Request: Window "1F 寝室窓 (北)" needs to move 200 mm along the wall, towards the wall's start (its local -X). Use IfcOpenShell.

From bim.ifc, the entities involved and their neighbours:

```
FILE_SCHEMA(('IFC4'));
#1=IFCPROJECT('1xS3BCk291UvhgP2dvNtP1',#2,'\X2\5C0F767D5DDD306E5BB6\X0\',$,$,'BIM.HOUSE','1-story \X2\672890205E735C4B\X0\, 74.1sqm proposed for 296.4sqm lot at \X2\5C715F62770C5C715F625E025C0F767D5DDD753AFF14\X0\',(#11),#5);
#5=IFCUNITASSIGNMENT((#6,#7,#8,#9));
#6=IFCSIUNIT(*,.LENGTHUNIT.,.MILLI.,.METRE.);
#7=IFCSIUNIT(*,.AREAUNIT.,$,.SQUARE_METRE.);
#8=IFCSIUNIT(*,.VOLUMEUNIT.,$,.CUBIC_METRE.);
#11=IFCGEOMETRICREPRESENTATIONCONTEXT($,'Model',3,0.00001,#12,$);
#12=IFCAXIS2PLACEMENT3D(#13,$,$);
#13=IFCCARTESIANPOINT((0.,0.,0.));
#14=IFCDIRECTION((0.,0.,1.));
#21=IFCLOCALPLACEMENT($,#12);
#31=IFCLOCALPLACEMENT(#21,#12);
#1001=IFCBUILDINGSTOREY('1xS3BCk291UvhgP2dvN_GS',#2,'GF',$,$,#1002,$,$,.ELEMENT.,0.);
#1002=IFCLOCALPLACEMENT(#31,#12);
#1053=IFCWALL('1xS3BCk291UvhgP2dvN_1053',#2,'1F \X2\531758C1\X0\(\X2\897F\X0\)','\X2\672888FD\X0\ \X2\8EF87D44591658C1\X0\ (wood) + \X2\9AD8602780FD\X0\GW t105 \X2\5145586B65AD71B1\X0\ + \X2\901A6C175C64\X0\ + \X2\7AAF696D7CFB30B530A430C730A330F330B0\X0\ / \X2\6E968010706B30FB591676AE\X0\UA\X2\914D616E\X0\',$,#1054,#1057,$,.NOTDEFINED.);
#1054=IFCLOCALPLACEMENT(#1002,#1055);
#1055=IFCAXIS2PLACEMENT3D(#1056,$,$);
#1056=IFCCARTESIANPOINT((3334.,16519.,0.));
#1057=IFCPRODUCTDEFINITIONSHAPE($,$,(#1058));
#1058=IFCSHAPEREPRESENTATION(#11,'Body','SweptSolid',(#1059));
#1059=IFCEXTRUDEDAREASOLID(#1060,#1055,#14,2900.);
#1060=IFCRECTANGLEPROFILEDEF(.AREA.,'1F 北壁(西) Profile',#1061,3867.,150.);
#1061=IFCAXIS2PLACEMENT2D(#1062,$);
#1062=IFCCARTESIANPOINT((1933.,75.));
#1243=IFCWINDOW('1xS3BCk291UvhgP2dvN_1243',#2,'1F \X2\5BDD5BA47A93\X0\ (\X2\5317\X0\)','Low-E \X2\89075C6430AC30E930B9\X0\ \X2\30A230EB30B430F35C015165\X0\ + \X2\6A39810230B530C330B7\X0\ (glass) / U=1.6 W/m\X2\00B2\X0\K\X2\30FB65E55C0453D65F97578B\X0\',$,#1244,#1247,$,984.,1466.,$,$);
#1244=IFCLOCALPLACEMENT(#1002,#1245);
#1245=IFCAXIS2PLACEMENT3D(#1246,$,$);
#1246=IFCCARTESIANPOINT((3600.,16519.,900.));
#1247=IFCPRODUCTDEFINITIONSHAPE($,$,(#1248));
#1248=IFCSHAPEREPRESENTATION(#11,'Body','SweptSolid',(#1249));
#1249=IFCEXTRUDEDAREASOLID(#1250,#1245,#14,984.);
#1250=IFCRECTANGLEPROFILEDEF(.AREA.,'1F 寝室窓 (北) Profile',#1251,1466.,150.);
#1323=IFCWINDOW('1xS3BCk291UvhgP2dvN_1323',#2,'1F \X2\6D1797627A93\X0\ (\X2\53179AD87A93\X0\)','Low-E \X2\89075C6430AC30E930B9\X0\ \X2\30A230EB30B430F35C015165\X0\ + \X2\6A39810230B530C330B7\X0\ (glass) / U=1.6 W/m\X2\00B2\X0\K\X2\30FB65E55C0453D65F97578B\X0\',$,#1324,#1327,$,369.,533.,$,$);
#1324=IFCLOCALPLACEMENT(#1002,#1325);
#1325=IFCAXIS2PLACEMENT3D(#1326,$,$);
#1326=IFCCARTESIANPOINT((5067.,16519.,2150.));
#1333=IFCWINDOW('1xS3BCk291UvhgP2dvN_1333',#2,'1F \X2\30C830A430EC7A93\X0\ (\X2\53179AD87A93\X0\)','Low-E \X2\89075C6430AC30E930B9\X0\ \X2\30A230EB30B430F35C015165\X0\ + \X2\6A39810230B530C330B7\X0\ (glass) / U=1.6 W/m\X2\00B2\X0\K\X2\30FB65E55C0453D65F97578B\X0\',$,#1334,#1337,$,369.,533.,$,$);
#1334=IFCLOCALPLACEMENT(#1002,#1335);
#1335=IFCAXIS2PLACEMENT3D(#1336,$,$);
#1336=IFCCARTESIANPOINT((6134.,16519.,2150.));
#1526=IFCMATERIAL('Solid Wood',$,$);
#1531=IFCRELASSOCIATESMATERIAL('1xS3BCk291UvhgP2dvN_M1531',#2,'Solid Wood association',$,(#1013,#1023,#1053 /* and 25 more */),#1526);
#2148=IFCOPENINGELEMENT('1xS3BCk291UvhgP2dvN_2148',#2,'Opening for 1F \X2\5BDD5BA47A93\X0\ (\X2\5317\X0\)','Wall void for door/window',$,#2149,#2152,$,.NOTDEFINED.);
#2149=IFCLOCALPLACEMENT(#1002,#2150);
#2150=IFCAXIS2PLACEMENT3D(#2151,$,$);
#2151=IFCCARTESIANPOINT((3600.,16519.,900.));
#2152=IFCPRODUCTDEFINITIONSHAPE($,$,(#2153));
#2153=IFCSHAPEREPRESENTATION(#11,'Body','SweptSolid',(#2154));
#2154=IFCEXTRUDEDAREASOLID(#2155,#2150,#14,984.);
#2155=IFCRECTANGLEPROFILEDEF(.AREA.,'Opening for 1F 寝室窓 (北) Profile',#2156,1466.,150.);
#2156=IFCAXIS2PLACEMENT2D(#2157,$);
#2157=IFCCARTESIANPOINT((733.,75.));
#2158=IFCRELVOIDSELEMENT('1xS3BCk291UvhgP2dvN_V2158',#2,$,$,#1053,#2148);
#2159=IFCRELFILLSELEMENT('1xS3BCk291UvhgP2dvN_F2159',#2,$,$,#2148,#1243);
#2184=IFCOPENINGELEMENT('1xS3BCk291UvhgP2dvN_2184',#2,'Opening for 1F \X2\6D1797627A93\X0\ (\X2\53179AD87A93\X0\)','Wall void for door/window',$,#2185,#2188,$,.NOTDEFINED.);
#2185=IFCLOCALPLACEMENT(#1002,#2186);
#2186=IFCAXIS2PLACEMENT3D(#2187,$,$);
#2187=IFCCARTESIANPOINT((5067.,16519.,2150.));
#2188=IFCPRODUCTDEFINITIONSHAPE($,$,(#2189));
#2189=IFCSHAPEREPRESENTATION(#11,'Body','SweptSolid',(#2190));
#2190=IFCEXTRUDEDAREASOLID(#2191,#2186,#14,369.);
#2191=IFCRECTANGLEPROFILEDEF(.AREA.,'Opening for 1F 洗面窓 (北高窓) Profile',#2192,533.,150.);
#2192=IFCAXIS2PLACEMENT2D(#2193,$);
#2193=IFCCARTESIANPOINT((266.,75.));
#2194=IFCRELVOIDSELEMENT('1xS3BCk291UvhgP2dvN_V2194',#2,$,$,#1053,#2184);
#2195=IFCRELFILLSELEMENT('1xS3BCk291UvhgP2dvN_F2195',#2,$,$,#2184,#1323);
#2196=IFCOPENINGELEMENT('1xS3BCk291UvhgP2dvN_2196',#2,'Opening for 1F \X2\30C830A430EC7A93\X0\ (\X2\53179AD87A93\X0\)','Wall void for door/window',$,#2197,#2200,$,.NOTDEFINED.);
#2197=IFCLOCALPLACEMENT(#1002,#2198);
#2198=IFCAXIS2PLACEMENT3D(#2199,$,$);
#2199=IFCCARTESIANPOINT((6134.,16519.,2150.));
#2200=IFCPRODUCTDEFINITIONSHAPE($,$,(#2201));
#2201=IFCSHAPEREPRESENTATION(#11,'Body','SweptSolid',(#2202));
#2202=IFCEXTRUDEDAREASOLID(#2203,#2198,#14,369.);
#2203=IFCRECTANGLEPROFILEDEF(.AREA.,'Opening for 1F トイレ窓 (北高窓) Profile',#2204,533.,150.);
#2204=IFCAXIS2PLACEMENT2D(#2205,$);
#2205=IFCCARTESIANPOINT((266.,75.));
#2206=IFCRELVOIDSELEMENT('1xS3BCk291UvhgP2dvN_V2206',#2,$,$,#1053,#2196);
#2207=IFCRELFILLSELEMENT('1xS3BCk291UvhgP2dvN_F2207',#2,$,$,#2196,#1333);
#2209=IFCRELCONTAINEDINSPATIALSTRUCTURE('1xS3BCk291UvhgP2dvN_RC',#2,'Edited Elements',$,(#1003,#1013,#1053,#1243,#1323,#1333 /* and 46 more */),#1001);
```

```python
import ifcopenshell
import ifcopenshell.api.geometry
import ifcopenshell.util.placement
import ifcopenshell.util.unit

model = ifcopenshell.open("bim.ifc")
unit_scale = ifcopenshell.util.unit.calculate_unit_scale(model)

window = model.by_guid("1xS3BCk291UvhgP2dvN_1243")
opening = window.FillsVoids[0].RelatingOpeningElement
wall = opening.VoidsElements[0].RelatingBuildingElement

wall_matrix = ifcopenshell.util.placement.get_local_placement(wall.ObjectPlacement)
shift = wall_matrix[:3, 0] * -0.2 / unit_scale
before = ifcopenshell.util.placement.get_local_placement(window.ObjectPlacement)[:3, 3].copy()

# The window is not placed relative to its opening, so move both.
for product in (opening, window):
    matrix = ifcopenshell.util.placement.get_local_placement(product.ObjectPlacement)
    matrix[:3, 3] += shift
    ifcopenshell.api.geometry.edit_object_placement(model, product=product, matrix=matrix, is_si=False)

after = ifcopenshell.util.placement.get_local_placement(window.ObjectPlacement)[:3, 3]
print("window moved by", (after - before).round(3) + 0.0)

model.write("bim_updated.ifc")
```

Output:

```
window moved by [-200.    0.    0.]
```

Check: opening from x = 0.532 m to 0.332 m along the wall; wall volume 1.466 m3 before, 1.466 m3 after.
